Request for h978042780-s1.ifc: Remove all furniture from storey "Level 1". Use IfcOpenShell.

First a look at what the model holds.

```python
import ifcopenshell
import ifcopenshell.util.element

model = ifcopenshell.open("h978042780-s1.ifc")
print(model.schema)
storey = next(s for s in model.by_type("IfcBuildingStorey") if s.Name == "Level 1")
furniture = [e for e in ifcopenshell.util.element.get_decomposition(storey) if e.is_a("IfcFurnishingElement")]
seen = {}
for e in furniture:
    element_type = ifcopenshell.util.element.get_type(e)
    name = element_type.Name if element_type not in (None, e) else None
    seen[name] = seen.get(name, 0) + 1
for name, count in sorted(seen.items(), key=str):
    print(count, "x", name)
```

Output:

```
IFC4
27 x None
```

```python
import ifcopenshell
import ifcopenshell.api.root
import ifcopenshell.util.element

model = ifcopenshell.open("h978042780-s1.ifc")

storey = next(s for s in model.by_type("IfcBuildingStorey") if s.Name == "Level 1")
furniture = [e for e in ifcopenshell.util.element.get_decomposition(storey) if e.is_a("IfcFurnishingElement")]

for e in furniture:
    ifcopenshell.api.root.remove_product(model, product=e)
print(len(furniture), "removed")

model.write("h978042780-s1_v2.ifc")
```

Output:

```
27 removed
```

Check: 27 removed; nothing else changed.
